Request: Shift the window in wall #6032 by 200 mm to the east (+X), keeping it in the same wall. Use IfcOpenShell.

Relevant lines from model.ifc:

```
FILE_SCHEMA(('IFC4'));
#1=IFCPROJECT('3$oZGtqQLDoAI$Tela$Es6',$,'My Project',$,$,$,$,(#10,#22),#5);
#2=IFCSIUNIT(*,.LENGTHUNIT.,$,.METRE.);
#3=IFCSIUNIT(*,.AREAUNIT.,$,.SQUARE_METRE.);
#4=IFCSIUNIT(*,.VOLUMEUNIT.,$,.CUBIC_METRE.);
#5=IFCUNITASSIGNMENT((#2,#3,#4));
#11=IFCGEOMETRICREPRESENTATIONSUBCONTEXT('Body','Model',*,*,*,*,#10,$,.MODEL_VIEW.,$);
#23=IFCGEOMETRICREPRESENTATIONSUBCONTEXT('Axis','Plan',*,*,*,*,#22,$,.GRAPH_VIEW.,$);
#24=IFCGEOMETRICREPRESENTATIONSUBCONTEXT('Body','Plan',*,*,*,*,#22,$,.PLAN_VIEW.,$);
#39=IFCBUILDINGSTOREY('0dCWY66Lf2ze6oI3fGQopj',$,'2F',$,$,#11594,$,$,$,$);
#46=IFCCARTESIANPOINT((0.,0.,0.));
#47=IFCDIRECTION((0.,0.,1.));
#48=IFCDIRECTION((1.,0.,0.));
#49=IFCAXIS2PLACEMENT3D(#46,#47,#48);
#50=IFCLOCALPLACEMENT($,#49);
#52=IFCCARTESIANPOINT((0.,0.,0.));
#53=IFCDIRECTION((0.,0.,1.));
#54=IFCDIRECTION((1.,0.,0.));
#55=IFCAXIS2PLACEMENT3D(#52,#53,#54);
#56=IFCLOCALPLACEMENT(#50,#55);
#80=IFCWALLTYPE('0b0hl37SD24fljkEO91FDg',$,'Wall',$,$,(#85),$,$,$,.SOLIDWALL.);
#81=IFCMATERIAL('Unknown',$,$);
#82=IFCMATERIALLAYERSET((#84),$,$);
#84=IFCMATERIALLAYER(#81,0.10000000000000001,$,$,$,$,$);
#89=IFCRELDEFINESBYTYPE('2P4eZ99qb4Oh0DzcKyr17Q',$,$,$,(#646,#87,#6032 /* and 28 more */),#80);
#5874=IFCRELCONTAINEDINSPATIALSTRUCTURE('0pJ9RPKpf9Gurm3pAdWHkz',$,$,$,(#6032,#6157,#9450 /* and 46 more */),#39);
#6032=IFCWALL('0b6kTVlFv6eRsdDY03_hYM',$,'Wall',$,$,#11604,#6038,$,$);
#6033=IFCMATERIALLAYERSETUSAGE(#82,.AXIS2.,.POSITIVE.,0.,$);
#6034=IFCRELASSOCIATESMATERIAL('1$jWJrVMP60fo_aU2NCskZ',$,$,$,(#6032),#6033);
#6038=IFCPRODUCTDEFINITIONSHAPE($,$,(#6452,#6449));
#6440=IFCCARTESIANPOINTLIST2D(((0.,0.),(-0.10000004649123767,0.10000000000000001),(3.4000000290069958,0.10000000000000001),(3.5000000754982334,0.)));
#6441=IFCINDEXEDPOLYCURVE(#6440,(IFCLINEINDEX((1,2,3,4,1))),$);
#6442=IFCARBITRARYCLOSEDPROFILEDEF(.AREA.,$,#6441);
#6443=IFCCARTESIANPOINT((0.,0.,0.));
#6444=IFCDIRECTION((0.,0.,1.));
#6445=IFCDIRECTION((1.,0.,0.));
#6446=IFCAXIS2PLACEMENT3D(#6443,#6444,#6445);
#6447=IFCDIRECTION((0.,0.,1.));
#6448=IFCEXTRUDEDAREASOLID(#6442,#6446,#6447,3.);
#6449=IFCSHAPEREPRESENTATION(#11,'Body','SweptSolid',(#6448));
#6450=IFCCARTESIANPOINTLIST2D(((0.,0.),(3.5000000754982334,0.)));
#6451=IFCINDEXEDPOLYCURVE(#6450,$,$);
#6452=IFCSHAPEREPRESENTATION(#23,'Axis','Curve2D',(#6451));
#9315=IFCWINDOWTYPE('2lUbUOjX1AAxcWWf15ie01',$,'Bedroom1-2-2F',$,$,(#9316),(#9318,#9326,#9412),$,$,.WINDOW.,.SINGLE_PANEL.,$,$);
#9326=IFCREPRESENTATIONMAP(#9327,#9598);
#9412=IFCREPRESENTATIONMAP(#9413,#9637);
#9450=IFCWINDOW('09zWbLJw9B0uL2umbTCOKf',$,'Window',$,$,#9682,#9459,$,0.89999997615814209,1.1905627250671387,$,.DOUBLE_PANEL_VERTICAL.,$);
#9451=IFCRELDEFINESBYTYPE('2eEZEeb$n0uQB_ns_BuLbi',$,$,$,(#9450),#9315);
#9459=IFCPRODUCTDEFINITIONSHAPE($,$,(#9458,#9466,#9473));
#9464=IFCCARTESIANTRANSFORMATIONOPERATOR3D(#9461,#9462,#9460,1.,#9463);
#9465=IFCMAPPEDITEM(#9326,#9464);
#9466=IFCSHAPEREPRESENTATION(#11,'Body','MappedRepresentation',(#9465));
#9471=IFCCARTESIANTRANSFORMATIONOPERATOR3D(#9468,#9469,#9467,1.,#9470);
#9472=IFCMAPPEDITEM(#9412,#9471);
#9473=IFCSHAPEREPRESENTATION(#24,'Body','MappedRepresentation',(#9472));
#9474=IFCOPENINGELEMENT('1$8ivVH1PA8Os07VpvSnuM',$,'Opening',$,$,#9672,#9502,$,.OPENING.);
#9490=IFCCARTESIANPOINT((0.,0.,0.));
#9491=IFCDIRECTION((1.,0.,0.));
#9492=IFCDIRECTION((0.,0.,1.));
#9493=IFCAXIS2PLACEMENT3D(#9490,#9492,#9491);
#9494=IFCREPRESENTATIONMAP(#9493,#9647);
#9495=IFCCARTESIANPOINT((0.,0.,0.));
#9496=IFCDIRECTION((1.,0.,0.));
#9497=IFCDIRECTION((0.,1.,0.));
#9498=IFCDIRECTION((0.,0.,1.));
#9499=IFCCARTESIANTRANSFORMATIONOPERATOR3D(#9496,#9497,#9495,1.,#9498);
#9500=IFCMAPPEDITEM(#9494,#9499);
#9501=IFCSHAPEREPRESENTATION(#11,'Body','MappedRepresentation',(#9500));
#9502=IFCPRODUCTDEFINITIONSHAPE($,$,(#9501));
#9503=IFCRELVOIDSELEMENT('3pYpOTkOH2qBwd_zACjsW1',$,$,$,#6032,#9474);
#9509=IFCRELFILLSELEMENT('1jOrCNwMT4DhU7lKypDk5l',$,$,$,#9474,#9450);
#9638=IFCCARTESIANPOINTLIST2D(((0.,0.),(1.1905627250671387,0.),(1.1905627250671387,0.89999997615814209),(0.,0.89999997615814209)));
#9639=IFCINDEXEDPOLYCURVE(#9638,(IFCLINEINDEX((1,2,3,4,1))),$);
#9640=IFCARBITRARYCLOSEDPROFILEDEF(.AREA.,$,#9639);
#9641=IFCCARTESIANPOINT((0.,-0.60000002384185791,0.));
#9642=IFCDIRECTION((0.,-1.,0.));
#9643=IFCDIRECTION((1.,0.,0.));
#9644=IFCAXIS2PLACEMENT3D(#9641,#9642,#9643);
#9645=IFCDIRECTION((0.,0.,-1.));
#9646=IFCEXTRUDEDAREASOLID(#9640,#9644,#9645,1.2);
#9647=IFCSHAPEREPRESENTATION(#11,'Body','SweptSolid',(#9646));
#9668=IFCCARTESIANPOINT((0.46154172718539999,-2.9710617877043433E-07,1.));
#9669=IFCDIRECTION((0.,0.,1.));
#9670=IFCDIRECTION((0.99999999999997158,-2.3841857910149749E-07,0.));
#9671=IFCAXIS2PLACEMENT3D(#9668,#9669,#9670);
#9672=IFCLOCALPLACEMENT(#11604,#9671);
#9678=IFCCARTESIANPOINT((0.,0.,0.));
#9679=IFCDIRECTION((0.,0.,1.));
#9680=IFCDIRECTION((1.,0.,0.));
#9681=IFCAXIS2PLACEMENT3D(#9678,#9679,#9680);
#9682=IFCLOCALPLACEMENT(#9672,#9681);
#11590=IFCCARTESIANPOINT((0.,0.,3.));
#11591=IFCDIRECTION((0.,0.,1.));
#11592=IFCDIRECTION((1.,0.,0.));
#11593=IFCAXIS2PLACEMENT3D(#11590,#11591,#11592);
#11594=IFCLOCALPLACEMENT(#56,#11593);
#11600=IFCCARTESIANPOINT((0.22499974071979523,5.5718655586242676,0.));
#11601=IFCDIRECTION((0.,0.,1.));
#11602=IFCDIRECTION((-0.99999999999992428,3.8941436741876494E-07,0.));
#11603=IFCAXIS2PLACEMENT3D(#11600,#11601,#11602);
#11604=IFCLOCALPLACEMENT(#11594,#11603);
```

```python
import ifcopenshell
import ifcopenshell.api.geometry
import ifcopenshell.util.placement

model = ifcopenshell.open("model.ifc")

window = model.by_guid("09zWbLJw9B0uL2umbTCOKf")
opening = window.FillsVoids[0].RelatingOpeningElement
wall = opening.VoidsElements[0].RelatingBuildingElement

wall_matrix = ifcopenshell.util.placement.get_local_placement(wall.ObjectPlacement)
shift = wall_matrix[:3, 0] * -0.2
before = ifcopenshell.util.placement.get_local_placement(window.ObjectPlacement)[:3, 3].copy()

# The window is placed relative to its opening, so it follows when the opening moves.
matrix = ifcopenshell.util.placement.get_local_placement(opening.ObjectPlacement)
matrix[:3, 3] += shift
ifcopenshell.api.geometry.edit_object_placement(
    model, product=opening, matrix=matrix, is_si=False, should_transform_children=True
)

after = ifcopenshell.util.placement.get_local_placement(window.ObjectPlacement)[:3, 3]
print("window moved by", (after - before).round(3) + 0.0)

model.write("model-out.ifc")
```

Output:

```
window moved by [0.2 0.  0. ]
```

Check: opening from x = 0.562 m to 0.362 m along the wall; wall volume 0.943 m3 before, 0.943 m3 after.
